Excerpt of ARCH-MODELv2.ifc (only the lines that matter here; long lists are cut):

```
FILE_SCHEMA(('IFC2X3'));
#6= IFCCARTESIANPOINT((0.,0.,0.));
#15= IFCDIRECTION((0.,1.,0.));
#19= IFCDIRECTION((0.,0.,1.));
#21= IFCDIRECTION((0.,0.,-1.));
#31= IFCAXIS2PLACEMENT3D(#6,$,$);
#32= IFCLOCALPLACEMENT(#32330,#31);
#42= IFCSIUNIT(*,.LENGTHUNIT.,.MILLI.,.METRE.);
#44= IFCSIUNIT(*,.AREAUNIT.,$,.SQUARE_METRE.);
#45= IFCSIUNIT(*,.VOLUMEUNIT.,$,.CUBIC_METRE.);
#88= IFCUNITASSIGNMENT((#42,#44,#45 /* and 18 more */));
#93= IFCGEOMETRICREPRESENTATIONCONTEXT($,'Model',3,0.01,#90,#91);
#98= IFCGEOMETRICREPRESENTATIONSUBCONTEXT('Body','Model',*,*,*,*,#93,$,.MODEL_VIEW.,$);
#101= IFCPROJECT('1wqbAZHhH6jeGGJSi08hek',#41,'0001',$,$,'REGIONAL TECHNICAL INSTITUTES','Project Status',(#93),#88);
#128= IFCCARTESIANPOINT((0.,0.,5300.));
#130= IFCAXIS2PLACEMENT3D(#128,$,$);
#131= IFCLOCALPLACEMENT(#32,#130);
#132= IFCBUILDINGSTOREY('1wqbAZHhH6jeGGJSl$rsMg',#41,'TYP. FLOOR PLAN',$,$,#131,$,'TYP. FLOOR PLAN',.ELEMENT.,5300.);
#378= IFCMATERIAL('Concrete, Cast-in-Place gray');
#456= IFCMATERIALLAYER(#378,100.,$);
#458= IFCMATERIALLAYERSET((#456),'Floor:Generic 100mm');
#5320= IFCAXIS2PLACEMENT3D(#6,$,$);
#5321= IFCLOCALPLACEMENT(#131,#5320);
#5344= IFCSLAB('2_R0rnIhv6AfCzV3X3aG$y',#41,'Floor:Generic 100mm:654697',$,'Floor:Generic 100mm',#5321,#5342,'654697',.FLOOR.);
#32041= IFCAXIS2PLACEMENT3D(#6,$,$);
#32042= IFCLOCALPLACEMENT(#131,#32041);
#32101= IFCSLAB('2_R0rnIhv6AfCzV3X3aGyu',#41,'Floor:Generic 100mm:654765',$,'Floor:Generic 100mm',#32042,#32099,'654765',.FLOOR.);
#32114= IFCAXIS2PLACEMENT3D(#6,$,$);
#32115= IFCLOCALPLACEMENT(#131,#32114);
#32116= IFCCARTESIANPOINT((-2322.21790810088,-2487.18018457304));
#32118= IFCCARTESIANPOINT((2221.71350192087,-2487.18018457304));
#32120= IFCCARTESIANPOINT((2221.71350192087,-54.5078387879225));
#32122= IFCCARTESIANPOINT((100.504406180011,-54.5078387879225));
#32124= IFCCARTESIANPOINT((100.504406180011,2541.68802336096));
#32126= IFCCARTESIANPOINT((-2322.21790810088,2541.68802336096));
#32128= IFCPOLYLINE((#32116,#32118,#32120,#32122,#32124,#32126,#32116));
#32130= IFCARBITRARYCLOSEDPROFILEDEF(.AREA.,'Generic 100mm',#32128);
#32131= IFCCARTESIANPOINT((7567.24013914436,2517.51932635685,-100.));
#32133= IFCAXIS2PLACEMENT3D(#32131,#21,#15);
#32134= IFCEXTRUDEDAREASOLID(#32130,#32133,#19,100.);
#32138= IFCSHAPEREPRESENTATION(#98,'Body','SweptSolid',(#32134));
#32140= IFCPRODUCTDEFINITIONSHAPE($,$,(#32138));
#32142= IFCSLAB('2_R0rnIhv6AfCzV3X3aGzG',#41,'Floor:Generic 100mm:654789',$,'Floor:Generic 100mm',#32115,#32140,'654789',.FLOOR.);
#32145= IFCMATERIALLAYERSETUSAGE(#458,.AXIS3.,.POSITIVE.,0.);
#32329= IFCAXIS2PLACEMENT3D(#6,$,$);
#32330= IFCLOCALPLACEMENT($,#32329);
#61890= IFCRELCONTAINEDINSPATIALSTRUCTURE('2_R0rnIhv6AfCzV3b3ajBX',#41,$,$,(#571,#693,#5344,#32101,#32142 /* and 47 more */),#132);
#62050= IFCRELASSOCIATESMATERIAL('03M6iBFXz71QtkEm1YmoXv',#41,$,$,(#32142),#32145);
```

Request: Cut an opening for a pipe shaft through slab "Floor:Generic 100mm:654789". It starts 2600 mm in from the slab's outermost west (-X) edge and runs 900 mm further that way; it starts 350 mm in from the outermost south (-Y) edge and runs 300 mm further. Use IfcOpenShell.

```python
import numpy as np
import ifcopenshell
import ifcopenshell.api.feature
import ifcopenshell.api.geometry
import ifcopenshell.api.root
import ifcopenshell.geom
import ifcopenshell.util.placement
import ifcopenshell.util.representation
import ifcopenshell.util.shape
import ifcopenshell.util.unit

model = ifcopenshell.open("ARCH-MODELv2.ifc")
unit_scale = ifcopenshell.util.unit.calculate_unit_scale(model)
settings = ifcopenshell.geom.settings()


def volume(element):
    """Net volume in cubic metres, openings subtracted."""
    shape = ifcopenshell.geom.create_shape(settings, element)
    return ifcopenshell.util.shape.get_volume(shape.geometry)


slab = model.by_guid("2_R0rnIhv6AfCzV3X3aGzG")
before = volume(slab)

# Extent in the slab's own axes, in metres. The edges named are its -X and -Y sides.
slab_shape = ifcopenshell.geom.create_shape(settings, slab)
vertices = ifcopenshell.util.shape.get_vertices(slab_shape.geometry)
x_min, y_min, bottom = vertices.min(axis=0)
top = vertices[:, 2].max()

opening = ifcopenshell.api.root.create_entity(model, ifc_class="IfcOpeningElement", name="Pipe shaft opening")
context = ifcopenshell.util.representation.get_context(model, "Model", "Body", "MODEL_VIEW")
width, depth = 0.9, 0.3
outline = [(0.0, 0.0), (width, 0.0), (width, depth), (0.0, depth), (0.0, 0.0)]
# Overshoot both faces by 50 mm so the cut is clean.
shape = ifcopenshell.api.geometry.add_slab_representation(
    model, context=context, depth=top - bottom + 0.1, polyline=outline
)
ifcopenshell.api.geometry.assign_representation(model, product=opening, representation=shape)

matrix = ifcopenshell.util.placement.get_local_placement(slab.ObjectPlacement)
matrix[:, 3] = matrix @ np.append(np.array([x_min + 2.6, y_min + 0.35, bottom - 0.05]) / unit_scale, 1.0)
ifcopenshell.api.geometry.edit_object_placement(model, product=opening, matrix=matrix, is_si=False)
ifcopenshell.api.feature.add_feature(model, feature=opening, element=slab)

after = volume(slab)

print(f"slab volume {before:.3f} -> {after:.3f} m3")

model.write("ARCH-MODELv2_updated.ifc")
```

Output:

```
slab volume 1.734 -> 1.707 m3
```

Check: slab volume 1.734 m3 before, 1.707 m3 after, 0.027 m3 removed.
